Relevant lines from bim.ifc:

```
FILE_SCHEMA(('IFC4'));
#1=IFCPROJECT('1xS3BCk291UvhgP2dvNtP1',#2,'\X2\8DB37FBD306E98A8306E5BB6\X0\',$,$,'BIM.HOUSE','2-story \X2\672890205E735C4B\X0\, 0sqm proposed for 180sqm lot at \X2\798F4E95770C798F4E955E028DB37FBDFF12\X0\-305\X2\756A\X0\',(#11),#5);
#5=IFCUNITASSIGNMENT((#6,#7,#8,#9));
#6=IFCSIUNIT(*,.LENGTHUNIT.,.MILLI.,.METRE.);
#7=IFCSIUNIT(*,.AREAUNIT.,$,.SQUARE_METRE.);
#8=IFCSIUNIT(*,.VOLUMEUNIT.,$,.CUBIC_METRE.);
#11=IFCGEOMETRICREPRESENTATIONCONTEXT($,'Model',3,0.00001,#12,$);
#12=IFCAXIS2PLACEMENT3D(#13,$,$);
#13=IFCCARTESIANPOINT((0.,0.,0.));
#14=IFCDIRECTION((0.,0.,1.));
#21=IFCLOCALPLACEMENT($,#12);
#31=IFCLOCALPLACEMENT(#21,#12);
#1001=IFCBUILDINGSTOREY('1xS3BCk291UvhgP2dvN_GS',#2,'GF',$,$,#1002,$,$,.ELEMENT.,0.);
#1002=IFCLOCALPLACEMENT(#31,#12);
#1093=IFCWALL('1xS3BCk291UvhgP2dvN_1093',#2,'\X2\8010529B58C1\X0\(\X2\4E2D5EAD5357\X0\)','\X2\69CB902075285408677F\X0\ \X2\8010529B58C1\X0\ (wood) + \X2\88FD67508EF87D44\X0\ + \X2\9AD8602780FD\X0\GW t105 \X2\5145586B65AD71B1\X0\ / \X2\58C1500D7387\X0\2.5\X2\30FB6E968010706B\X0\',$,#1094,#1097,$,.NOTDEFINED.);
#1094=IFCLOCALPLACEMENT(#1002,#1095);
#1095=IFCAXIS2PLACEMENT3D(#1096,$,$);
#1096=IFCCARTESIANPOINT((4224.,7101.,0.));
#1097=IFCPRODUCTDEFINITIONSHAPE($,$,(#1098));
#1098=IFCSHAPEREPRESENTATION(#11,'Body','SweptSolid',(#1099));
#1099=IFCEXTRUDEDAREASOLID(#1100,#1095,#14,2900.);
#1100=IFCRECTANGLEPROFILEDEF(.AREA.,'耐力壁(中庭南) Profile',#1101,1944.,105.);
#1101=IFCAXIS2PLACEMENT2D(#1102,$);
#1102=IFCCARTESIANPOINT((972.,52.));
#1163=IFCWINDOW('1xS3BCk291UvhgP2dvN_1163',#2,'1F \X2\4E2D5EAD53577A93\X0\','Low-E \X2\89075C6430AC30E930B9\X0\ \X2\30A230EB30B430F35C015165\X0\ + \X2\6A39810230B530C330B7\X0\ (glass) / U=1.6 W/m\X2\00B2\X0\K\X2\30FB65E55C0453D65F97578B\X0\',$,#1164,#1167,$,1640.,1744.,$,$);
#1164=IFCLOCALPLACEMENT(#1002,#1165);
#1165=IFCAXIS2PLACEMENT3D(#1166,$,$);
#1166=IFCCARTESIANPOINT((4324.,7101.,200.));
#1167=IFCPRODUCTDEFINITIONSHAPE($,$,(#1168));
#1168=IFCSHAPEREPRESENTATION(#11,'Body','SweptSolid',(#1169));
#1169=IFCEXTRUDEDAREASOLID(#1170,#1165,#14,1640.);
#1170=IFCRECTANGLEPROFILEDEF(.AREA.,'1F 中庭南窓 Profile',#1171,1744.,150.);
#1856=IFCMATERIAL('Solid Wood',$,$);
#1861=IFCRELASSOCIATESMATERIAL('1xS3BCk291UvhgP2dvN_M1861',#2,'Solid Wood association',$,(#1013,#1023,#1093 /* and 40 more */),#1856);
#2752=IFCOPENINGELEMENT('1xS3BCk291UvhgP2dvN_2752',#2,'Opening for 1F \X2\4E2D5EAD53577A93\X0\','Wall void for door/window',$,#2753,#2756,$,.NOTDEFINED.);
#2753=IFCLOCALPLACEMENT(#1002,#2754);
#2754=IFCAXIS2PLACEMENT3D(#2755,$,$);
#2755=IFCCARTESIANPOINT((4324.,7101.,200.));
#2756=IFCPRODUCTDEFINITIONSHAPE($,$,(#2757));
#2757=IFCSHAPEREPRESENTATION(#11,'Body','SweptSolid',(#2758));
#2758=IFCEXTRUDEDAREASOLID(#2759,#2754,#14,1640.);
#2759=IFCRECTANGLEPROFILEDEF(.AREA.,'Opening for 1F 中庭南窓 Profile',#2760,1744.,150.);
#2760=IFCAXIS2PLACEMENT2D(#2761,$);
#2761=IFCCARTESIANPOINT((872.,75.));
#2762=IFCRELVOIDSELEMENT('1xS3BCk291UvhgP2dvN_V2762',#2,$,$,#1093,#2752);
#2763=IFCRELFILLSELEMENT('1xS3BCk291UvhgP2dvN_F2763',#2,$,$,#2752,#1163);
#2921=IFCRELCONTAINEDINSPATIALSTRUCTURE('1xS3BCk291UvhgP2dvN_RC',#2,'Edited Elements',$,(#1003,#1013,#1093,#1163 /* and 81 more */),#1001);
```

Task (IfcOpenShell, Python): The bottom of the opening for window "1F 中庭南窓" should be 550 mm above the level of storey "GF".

```python
import numpy as np
import ifcopenshell
import ifcopenshell.api.geometry
import ifcopenshell.geom
import ifcopenshell.util.element
import ifcopenshell.util.placement
import ifcopenshell.util.shape
import ifcopenshell.util.unit

model = ifcopenshell.open("bim.ifc")
unit_scale = ifcopenshell.util.unit.calculate_unit_scale(model)

window = model.by_id(1163)
opening = window.FillsVoids[0].RelatingOpeningElement
storey = ifcopenshell.util.element.get_container(window, ifc_class="IfcBuildingStorey")
level = ifcopenshell.util.placement.get_local_placement(storey.ObjectPlacement)[2, 3]

# The opening's origin need not be at the sill, so measure its lowest point.
shape = ifcopenshell.geom.create_shape(ifcopenshell.geom.settings(), opening)
bottom = ifcopenshell.util.shape.get_shape_bottom_elevation(shape, shape.geometry) / unit_scale
dz = level + 550.0 - bottom

shift = np.array([0.0, 0.0, dz])
# The window is not placed relative to its opening, so move both.
for product in (opening, window):
    matrix = ifcopenshell.util.placement.get_local_placement(product.ObjectPlacement)
    matrix[:3, 3] += shift
    ifcopenshell.api.geometry.edit_object_placement(model, product=product, matrix=matrix, is_si=False)

print(f"moved by {dz * unit_scale:+.3f} m")

model.write("bim_v2.ifc")
```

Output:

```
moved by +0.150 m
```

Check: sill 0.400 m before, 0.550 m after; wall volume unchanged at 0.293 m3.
